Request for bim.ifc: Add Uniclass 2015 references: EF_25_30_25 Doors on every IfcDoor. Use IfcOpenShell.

First a look at what the model holds.

```python
import ifcopenshell

model = ifcopenshell.open("bim.ifc")
print(model.schema)
print("classifications:", [c.Name for c in model.by_type("IfcClassification")])
for ifc_class in ("IfcDoor", "IfcRoof", "IfcStair", "IfcWall", "IfcWindow"):
    print(ifc_class, len(model.by_type(ifc_class)))
```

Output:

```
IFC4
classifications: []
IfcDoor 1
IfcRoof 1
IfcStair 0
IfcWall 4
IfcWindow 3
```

```python
import ifcopenshell
import ifcopenshell.api.classification

model = ifcopenshell.open("bim.ifc")

system = ifcopenshell.api.classification.add_classification(model, classification="Uniclass 2015")

codes = {
    "IfcDoor": ("EF_25_30_25", "Doors"),
}
for ifc_class, (code, name) in codes.items():
    products = model.by_type(ifc_class)
    ifcopenshell.api.classification.add_reference(
        model, products=products, classification=system, identification=code, name=name
    )
    print(code, len(products))

model.write("bim_edited.ifc")
```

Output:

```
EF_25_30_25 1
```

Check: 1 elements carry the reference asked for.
